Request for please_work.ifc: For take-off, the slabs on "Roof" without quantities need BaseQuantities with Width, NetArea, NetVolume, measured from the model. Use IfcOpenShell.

First a look at what the model holds.

```python
import ifcopenshell
import ifcopenshell.util.element
import ifcopenshell.util.unit

model = ifcopenshell.open("please_work.ifc")
print(model.schema)
for unit_type in ("LENGTHUNIT", "AREAUNIT", "VOLUMEUNIT"):
    print(unit_type, ifcopenshell.util.unit.calculate_unit_scale(model, unit_type))
storey = next(s for s in model.by_type("IfcBuildingStorey") if s.Name == "Roof")
slabs = [e for e in ifcopenshell.util.element.get_decomposition(storey) if e.is_a("IfcSlab")]
for e in sorted(slabs, key=lambda e: e.id()):
    print(e.id(), e.is_a(), e.Name, list(ifcopenshell.util.element.get_psets(e, qtos_only=True)), sep=" | ")
```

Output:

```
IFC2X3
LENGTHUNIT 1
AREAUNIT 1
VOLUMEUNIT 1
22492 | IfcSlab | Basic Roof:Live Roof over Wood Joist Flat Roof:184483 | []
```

```python
import ifcopenshell
import ifcopenshell.api.pset
import ifcopenshell.geom
import ifcopenshell.util.element
import ifcopenshell.util.shape
import ifcopenshell.util.unit

model = ifcopenshell.open("please_work.ifc")
unit_scale = ifcopenshell.util.unit.calculate_unit_scale(model)
area_scale = ifcopenshell.util.unit.calculate_unit_scale(model, "AREAUNIT")
volume_scale = ifcopenshell.util.unit.calculate_unit_scale(model, "VOLUMEUNIT")
settings = ifcopenshell.geom.settings()

storey = next(s for s in model.by_type("IfcBuildingStorey") if s.Name == "Roof")
slabs = [e for e in ifcopenshell.util.element.get_decomposition(storey) if e.is_a("IfcSlab")]

for e in sorted(slabs, key=lambda e: e.id()):
    if ifcopenshell.util.element.get_psets(e, qtos_only=True, should_inherit=False):
        continue
    # Geometry comes back in metres, in the element's own axes.
    shape = ifcopenshell.geom.create_shape(settings, e)
    values = {
        "Width": ifcopenshell.util.shape.get_z(shape.geometry) / unit_scale,
        "NetArea": ifcopenshell.util.shape.get_footprint_area(shape.geometry) / area_scale,
        "NetVolume": ifcopenshell.util.shape.get_volume(shape.geometry) / volume_scale,
    }
    qto = ifcopenshell.api.pset.add_qto(model, product=e, name="BaseQuantities")
    ifcopenshell.api.pset.edit_qto(model, qto=qto, properties=values)
    print(e.id(), {k: round(v, 3) for k, v in values.items()})

model.write("please_work_v2.ifc")
```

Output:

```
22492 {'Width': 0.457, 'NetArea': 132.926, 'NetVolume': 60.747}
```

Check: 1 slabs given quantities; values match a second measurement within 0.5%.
